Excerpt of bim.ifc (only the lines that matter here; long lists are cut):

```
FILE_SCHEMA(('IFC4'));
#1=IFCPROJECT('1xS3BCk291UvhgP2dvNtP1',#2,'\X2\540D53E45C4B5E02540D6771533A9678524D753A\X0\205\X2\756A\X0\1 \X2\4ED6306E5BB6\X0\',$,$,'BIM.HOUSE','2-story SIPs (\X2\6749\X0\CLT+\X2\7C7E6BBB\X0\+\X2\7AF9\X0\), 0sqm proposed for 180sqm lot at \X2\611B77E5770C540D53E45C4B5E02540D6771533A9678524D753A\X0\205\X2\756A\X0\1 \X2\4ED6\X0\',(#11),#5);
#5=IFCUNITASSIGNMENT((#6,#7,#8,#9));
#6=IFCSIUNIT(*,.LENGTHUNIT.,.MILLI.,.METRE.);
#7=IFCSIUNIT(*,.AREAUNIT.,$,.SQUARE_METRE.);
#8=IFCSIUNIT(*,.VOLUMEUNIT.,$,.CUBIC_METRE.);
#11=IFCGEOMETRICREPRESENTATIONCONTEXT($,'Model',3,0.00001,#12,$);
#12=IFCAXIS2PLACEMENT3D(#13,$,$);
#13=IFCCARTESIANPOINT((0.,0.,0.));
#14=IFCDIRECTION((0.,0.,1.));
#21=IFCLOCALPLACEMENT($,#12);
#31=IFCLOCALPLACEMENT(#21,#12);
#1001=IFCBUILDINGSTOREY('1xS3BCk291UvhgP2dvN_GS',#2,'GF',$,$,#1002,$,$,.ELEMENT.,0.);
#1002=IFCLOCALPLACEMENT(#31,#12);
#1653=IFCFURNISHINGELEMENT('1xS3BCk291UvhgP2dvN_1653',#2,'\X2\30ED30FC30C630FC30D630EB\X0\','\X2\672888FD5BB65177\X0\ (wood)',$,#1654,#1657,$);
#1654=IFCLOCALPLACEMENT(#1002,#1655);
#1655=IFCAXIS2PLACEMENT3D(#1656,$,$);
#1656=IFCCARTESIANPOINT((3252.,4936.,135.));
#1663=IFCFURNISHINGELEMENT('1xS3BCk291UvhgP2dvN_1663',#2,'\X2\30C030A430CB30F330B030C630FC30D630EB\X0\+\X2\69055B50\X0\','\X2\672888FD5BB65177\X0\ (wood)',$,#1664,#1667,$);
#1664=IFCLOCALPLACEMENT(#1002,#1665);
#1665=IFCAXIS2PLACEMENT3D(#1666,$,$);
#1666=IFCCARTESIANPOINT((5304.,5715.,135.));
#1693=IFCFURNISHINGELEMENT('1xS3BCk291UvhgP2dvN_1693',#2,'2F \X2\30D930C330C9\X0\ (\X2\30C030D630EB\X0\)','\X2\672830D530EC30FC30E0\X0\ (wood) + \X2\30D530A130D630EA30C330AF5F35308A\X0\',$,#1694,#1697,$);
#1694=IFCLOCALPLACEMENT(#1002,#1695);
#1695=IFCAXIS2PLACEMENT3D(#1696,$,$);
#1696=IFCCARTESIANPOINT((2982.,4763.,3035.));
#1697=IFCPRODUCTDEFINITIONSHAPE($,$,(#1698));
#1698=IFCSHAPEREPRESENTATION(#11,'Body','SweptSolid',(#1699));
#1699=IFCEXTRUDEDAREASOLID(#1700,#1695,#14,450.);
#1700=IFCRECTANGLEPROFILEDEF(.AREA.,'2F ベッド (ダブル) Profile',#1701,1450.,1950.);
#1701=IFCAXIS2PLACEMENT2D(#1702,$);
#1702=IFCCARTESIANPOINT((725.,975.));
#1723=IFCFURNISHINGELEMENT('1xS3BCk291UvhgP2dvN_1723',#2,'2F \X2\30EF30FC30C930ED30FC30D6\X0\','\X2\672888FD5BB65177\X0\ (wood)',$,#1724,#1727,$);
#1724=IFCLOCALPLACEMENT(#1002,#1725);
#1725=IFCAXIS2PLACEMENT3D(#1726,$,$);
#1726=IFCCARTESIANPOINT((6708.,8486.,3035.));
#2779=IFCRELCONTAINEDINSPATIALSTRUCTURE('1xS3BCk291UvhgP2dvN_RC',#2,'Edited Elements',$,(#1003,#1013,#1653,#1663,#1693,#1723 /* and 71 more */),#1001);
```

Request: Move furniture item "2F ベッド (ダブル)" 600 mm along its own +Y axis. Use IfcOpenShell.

```python
import ifcopenshell
import ifcopenshell.api.geometry
import ifcopenshell.util.placement

model = ifcopenshell.open("bim.ifc")

item = model.by_id(1693)
matrix = ifcopenshell.util.placement.get_local_placement(item.ObjectPlacement)
matrix[:3, 3] += matrix[:3, 1] * 600.0
ifcopenshell.api.geometry.edit_object_placement(model, product=item, matrix=matrix, is_si=False)

print(ifcopenshell.util.placement.get_local_placement(item.ObjectPlacement).round(3) + 0.0)

model.write("bim-out.ifc")
```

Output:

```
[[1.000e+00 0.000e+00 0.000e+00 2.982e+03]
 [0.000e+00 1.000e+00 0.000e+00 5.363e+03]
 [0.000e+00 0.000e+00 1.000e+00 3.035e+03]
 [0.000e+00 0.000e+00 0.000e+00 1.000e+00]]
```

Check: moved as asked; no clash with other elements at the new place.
